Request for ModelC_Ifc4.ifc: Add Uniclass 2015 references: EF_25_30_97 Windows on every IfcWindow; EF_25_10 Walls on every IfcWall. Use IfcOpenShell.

First a look at what the model holds.

```python
import ifcopenshell

model = ifcopenshell.open("ModelC_Ifc4.ifc")
print(model.schema)
print("classifications:", [c.Name for c in model.by_type("IfcClassification")])
for ifc_class in ("IfcDoor", "IfcRoof", "IfcStair", "IfcWall", "IfcWindow"):
    print(ifc_class, len(model.by_type(ifc_class)))
```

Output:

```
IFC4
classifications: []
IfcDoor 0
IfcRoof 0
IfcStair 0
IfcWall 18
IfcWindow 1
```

```python
import ifcopenshell
import ifcopenshell.api.classification

model = ifcopenshell.open("ModelC_Ifc4.ifc")

system = ifcopenshell.api.classification.add_classification(model, classification="Uniclass 2015")

codes = {
    "IfcWindow": ("EF_25_30_97", "Windows"),
    "IfcWall": ("EF_25_10", "Walls"),
}
for ifc_class, (code, name) in codes.items():
    products = model.by_type(ifc_class)
    ifcopenshell.api.classification.add_reference(
        model, products=products, classification=system, identification=code, name=name
    )
    print(code, len(products))

model.write("ModelC_Ifc4_updated.ifc")
```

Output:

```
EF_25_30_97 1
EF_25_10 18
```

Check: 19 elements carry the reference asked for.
